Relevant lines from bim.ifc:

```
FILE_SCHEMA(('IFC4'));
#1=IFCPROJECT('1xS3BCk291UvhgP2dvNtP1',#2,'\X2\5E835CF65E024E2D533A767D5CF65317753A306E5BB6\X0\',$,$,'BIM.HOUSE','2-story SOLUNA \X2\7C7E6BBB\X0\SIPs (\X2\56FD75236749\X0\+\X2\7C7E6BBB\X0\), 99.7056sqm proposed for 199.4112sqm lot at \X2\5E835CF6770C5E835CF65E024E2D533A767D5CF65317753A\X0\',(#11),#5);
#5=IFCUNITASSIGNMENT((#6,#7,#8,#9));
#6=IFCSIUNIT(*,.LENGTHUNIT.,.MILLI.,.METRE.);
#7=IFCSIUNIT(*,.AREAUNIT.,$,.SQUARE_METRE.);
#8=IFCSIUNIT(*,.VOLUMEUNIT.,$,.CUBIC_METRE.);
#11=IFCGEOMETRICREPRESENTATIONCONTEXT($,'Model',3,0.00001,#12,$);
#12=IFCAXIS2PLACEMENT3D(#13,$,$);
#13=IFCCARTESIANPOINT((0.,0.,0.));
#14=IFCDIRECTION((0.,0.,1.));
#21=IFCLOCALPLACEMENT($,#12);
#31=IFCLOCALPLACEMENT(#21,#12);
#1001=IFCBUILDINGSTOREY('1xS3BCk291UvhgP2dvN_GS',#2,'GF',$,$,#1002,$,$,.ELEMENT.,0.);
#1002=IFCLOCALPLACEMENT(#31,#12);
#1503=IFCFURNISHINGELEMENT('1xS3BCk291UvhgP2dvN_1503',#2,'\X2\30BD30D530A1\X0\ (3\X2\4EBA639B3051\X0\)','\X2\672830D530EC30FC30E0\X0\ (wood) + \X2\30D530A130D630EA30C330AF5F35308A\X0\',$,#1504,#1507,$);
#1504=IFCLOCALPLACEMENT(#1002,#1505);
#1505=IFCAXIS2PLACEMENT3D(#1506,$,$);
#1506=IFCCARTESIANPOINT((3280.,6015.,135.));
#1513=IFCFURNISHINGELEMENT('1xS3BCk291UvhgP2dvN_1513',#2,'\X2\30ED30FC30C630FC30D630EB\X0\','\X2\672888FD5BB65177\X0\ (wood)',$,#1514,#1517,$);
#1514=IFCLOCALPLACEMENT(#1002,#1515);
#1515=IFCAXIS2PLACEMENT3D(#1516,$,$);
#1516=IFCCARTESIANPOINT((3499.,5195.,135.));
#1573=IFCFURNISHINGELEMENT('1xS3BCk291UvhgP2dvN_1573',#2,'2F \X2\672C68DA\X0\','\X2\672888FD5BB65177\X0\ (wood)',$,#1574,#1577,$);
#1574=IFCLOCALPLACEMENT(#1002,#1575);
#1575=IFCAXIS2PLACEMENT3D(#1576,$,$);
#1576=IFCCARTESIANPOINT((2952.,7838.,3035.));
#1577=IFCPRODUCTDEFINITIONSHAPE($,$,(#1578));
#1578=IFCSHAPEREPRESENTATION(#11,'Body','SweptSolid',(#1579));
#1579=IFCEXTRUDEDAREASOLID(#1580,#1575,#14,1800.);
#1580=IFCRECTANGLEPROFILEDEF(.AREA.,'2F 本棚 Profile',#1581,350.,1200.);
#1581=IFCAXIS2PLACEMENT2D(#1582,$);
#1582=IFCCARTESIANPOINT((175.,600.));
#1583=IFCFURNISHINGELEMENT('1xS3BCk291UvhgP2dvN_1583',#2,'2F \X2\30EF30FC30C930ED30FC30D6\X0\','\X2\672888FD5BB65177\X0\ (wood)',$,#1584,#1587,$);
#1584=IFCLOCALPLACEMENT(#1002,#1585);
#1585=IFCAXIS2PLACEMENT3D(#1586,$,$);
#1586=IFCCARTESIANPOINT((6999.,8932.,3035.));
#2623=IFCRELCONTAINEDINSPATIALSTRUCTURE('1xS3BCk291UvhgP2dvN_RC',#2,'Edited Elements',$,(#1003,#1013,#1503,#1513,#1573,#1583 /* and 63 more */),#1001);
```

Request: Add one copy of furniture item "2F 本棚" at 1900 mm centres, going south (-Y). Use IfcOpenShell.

```python
import numpy as np
import ifcopenshell
import ifcopenshell.api.geometry
import ifcopenshell.api.root
import ifcopenshell.util.element
import ifcopenshell.util.placement
import ifcopenshell.util.unit

model = ifcopenshell.open("bim.ifc")
unit_scale = ifcopenshell.util.unit.calculate_unit_scale(model)


def reuse_history(source, copy):
    """copy_class also copies each property set's owner history, people and application; keep the originals."""
    for rel in copy.IsDefinedBy:
        if rel.is_a("IfcRelDefinesByProperties") and (history := rel.RelatingPropertyDefinition.OwnerHistory):
            rel.RelatingPropertyDefinition.OwnerHistory = source.OwnerHistory
            ifcopenshell.util.element.remove_deep2(model, history)


source = model.by_id(1573)
base = ifcopenshell.util.placement.get_local_placement(source.ObjectPlacement)
step = np.array([0.0, -1.0, 0.0]) * 1.9 / unit_scale

for i in range(1, 2):
    copy = ifcopenshell.api.root.copy_class(model, product=source)
    copy.Representation = ifcopenshell.util.element.copy_deep(
        model, source.Representation, exclude=["IfcGeometricRepresentationContext", "IfcRepresentationMap"]
    )
    reuse_history(source, copy)
    matrix = base.copy()
    matrix[:3, 3] += i * step
    print("added at", matrix[:3, 3].round(3) + 0.0)
    ifcopenshell.api.geometry.edit_object_placement(model, product=copy, matrix=matrix, is_si=False)

model.write("bim_rev.ifc")
```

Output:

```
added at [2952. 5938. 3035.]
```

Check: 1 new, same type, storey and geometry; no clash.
